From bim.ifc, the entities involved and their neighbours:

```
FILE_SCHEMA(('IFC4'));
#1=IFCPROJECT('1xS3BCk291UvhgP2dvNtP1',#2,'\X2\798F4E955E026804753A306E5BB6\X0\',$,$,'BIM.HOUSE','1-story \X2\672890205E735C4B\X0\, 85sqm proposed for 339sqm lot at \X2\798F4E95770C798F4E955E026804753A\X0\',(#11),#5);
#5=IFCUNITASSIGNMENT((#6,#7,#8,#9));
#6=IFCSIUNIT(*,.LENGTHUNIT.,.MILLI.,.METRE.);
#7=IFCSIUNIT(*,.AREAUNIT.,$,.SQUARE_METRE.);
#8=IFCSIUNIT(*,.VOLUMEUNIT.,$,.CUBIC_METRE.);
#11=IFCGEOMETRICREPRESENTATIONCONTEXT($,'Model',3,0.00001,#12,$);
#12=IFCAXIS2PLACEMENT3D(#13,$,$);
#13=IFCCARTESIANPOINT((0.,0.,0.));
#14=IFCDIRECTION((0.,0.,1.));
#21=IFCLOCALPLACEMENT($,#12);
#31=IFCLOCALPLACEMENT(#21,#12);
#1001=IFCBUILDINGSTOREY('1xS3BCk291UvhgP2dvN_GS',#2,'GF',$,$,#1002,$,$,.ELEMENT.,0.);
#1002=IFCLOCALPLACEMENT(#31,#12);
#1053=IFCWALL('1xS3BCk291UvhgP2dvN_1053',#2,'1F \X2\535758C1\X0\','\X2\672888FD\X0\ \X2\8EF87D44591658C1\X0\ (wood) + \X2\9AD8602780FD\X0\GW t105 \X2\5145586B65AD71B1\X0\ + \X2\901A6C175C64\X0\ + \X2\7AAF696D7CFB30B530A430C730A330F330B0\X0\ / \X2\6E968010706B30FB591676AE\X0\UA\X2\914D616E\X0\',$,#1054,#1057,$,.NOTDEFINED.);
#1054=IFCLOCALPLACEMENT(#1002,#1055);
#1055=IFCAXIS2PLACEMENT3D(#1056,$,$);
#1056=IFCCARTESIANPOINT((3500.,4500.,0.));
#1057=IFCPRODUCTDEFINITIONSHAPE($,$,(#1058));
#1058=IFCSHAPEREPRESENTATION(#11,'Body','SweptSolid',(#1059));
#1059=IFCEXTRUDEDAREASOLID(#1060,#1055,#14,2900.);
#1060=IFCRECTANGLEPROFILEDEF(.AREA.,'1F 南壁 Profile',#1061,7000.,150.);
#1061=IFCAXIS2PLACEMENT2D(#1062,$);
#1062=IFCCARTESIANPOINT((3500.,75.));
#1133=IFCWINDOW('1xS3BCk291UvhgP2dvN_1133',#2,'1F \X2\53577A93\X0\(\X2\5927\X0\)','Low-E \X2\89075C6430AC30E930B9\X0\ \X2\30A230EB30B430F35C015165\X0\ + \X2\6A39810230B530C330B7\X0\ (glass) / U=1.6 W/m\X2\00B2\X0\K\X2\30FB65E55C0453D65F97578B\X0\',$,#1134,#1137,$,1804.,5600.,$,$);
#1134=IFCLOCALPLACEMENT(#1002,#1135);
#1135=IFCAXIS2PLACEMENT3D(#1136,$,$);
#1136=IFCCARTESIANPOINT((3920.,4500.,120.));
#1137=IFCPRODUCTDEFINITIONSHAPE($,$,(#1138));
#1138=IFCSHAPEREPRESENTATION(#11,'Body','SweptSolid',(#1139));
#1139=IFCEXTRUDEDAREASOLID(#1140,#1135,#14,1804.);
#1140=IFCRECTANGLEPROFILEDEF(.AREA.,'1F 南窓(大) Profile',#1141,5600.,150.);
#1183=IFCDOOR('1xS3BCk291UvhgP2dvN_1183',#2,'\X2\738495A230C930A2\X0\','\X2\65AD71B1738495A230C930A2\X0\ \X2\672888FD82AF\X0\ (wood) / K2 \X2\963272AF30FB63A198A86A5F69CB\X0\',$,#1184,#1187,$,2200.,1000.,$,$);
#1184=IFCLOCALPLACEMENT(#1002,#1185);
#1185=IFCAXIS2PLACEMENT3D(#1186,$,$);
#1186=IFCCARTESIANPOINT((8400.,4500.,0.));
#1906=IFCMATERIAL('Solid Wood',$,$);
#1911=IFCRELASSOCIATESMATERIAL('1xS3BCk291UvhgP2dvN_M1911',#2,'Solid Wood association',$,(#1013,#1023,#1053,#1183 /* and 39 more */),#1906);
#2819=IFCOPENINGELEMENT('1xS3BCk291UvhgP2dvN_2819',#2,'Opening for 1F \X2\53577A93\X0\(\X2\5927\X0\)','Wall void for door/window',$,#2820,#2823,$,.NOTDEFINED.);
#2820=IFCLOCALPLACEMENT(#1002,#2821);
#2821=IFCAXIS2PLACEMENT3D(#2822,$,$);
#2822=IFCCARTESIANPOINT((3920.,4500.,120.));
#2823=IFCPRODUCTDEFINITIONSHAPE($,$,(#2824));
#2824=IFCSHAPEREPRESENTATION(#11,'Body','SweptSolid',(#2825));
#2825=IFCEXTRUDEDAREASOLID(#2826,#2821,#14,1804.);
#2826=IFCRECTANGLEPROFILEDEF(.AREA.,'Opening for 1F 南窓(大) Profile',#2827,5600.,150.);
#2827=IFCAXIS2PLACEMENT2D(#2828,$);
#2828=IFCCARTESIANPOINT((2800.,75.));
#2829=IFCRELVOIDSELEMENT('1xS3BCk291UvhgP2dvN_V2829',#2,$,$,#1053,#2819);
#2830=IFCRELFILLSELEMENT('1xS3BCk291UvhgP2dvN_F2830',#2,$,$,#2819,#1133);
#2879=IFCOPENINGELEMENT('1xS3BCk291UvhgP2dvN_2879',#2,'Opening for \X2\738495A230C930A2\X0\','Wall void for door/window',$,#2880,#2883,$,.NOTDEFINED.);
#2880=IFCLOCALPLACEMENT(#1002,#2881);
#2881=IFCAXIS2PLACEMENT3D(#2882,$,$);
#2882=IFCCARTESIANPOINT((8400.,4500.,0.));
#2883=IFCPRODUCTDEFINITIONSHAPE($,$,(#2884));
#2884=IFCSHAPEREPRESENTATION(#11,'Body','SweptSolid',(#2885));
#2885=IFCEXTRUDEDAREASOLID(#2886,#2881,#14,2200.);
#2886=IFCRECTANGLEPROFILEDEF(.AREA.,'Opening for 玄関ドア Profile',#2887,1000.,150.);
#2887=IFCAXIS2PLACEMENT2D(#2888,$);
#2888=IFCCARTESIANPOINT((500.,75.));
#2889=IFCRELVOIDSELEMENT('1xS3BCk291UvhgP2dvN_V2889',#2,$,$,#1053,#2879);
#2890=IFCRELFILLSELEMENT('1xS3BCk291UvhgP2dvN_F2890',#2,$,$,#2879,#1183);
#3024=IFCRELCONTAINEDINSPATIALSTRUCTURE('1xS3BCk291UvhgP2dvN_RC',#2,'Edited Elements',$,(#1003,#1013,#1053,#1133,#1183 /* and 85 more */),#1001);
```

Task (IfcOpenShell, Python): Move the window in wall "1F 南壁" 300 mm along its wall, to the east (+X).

```python
import ifcopenshell
import ifcopenshell.api.geometry
import ifcopenshell.util.placement

model = ifcopenshell.open("bim.ifc")

window = model.by_id(1133)
opening = window.FillsVoids[0].RelatingOpeningElement
wall = opening.VoidsElements[0].RelatingBuildingElement

wall_matrix = ifcopenshell.util.placement.get_local_placement(wall.ObjectPlacement)
shift = wall_matrix[:3, 0] * 300.0
before = ifcopenshell.util.placement.get_local_placement(window.ObjectPlacement)[:3, 3].copy()

# The window is not placed relative to its opening, so move both.
for product in (opening, window):
    matrix = ifcopenshell.util.placement.get_local_placement(product.ObjectPlacement)
    matrix[:3, 3] += shift
    ifcopenshell.api.geometry.edit_object_placement(model, product=product, matrix=matrix, is_si=False)

after = ifcopenshell.util.placement.get_local_placement(window.ObjectPlacement)[:3, 3]
print("window moved by", (after - before).round(3) + 0.0)

model.write("bim_v2.ifc")
```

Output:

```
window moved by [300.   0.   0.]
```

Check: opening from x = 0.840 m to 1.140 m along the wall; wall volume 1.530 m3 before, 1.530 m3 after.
